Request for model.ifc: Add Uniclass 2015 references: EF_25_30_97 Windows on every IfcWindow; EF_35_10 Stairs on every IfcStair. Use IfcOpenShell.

First a look at what the model holds.

```python
import ifcopenshell

model = ifcopenshell.open("model.ifc")
print(model.schema)
print("classifications:", [c.Name for c in model.by_type("IfcClassification")])
for ifc_class in ("IfcDoor", "IfcRoof", "IfcStair", "IfcWall", "IfcWindow"):
    print(ifc_class, len(model.by_type(ifc_class)))
```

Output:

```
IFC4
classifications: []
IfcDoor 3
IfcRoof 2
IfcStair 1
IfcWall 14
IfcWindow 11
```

```python
import ifcopenshell
import ifcopenshell.api.classification

model = ifcopenshell.open("model.ifc")

system = ifcopenshell.api.classification.add_classification(model, classification="Uniclass 2015")

codes = {
    "IfcWindow": ("EF_25_30_97", "Windows"),
    "IfcStair": ("EF_35_10", "Stairs"),
}
for ifc_class, (code, name) in codes.items():
    products = model.by_type(ifc_class)
    ifcopenshell.api.classification.add_reference(
        model, products=products, classification=system, identification=code, name=name
    )
    print(code, len(products))

model.write("model_edited.ifc")
```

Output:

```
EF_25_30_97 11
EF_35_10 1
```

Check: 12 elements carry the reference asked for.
